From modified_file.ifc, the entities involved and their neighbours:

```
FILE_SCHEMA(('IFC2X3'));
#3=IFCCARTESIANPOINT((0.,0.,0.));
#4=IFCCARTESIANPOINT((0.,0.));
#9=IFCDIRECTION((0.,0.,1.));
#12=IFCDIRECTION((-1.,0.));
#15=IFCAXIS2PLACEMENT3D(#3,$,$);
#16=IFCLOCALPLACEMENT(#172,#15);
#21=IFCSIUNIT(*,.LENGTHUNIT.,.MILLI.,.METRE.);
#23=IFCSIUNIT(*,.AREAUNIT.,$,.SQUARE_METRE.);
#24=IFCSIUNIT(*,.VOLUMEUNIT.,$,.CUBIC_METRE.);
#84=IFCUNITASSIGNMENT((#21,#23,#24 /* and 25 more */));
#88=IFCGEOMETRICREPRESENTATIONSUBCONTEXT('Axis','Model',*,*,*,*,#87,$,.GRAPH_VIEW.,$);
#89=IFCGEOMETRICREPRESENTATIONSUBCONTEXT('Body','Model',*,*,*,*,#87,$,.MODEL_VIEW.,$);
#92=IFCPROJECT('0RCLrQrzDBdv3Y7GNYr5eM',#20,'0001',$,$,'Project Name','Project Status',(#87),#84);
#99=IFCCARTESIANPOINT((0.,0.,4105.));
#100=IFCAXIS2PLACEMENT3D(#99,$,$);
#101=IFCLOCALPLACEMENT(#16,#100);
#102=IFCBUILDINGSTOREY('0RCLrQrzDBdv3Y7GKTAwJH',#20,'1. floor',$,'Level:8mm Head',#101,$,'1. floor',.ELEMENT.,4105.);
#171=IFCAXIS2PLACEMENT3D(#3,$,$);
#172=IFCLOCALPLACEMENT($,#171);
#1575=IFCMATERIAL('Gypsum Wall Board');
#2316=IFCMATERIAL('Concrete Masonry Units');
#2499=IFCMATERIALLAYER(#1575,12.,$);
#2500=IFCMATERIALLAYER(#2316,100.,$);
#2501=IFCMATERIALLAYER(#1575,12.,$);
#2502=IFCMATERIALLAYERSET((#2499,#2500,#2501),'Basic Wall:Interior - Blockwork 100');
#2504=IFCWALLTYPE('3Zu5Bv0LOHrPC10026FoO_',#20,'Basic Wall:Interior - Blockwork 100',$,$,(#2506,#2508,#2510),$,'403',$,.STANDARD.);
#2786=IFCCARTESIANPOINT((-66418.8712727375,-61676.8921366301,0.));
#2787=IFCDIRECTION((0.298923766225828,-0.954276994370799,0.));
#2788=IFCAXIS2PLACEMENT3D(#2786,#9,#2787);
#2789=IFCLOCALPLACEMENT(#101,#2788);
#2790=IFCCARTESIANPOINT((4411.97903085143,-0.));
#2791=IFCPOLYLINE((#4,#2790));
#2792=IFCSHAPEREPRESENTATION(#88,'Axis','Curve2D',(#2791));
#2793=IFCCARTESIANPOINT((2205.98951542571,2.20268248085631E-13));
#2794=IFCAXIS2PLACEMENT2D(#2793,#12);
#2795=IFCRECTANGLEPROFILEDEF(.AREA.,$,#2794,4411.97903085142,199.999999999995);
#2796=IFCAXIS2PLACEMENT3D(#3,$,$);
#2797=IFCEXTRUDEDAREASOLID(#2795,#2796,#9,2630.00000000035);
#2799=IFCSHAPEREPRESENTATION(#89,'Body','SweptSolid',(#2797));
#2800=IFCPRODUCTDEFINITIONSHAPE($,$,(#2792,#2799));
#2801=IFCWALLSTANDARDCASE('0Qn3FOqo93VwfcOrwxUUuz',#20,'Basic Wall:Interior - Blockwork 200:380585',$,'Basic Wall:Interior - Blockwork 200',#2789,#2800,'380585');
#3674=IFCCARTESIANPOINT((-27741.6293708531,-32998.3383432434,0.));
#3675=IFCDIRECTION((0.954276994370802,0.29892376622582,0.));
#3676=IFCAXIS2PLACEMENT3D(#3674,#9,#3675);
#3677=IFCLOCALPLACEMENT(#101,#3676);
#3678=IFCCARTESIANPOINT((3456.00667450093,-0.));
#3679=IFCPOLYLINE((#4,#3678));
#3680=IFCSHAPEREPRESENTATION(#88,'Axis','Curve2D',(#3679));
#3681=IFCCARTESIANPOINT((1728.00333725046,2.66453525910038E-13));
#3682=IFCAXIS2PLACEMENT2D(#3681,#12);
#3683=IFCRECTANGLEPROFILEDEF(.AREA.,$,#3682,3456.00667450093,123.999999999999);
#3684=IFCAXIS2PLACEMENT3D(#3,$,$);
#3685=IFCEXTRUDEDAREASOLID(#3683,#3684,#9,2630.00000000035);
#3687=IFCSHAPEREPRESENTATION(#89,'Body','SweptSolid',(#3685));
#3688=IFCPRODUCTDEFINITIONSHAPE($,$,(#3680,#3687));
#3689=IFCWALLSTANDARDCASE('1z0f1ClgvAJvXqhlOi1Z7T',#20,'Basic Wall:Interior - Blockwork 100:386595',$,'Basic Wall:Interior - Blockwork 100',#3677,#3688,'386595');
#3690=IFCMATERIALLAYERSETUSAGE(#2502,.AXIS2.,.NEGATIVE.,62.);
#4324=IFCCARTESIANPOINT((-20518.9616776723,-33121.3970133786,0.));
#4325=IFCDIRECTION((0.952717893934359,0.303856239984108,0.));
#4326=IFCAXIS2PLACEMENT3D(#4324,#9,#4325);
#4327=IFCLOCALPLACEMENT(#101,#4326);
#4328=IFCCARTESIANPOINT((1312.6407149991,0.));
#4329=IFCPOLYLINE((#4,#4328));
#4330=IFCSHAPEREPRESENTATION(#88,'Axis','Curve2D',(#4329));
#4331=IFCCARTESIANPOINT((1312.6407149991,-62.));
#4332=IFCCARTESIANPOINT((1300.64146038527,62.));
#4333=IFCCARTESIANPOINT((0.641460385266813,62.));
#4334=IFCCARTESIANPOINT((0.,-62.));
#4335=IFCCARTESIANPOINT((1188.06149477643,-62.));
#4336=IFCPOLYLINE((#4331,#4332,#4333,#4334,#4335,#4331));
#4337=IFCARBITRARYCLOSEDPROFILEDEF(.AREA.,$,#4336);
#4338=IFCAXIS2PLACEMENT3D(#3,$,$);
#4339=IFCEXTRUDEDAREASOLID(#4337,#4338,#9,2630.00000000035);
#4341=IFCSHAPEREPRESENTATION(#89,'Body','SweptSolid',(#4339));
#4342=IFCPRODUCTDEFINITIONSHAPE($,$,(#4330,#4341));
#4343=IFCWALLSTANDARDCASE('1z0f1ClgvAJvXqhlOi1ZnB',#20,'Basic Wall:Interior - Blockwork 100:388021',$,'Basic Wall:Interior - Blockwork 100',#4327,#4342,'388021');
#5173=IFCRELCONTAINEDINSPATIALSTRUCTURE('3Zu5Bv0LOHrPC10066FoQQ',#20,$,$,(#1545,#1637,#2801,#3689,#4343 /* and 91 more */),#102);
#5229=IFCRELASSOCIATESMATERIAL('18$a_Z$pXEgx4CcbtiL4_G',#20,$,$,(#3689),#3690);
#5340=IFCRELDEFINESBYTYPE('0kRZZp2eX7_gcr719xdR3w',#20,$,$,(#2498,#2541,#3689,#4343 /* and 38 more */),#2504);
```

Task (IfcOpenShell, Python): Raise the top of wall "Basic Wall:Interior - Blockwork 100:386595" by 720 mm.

```python
import ifcopenshell
import ifcopenshell.geom
import ifcopenshell.util.representation
import ifcopenshell.util.shape
import ifcopenshell.util.unit

model = ifcopenshell.open("modified_file.ifc")
unit_scale = ifcopenshell.util.unit.calculate_unit_scale(model)
settings = ifcopenshell.geom.settings()


def volume(element):
    """Net volume in cubic metres, openings subtracted."""
    shape = ifcopenshell.geom.create_shape(settings, element)
    return ifcopenshell.util.shape.get_volume(shape.geometry)


wall = model.by_id(3689)
before = volume(wall)

body = ifcopenshell.util.representation.get_representation(wall, "Model", "Body")
solid = body.Items[0]
old_height = solid.Depth
solid.Depth += 0.72 / unit_scale
after = volume(wall)

print(f"height {old_height:g} -> {solid.Depth:g}, volume {before:.3f} -> {after:.3f} m3")

model.write("modified_file_rev.ifc")
```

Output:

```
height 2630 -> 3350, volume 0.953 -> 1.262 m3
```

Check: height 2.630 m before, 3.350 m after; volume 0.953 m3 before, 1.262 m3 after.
